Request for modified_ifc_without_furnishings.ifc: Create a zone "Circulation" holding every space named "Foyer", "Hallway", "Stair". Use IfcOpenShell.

First a look at what the model holds.

```python
import ifcopenshell

model = ifcopenshell.open("modified_ifc_without_furnishings.ifc")
print(model.schema)
seen = {}
for space in model.by_type("IfcSpace"):
    seen[space.LongName] = seen.get(space.LongName, 0) + 1
for name, count in sorted(seen.items(), key=str):
    print(count, "x", name)
print("zones:", [z.Name for z in model.by_type("IfcZone")][:20])
```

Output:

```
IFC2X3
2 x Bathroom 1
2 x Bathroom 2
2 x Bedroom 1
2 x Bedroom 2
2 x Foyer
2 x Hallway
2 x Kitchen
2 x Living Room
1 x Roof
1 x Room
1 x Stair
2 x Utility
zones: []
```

```python
import ifcopenshell
import ifcopenshell.api.group
import ifcopenshell.api.root

model = ifcopenshell.open("modified_ifc_without_furnishings.ifc")

names = {"Foyer", "Hallway", "Stair"}
spaces = [s for s in model.by_type("IfcSpace") if s.LongName in names]

zone = ifcopenshell.api.root.create_entity(model, ifc_class="IfcZone", name="Circulation")
ifcopenshell.api.group.assign_group(model, products=spaces, group=zone)
print(len(spaces), "spaces in", zone.Name)

model.write("modified_ifc_without_furnishings_v2.ifc")
```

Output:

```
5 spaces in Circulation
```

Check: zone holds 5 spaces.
